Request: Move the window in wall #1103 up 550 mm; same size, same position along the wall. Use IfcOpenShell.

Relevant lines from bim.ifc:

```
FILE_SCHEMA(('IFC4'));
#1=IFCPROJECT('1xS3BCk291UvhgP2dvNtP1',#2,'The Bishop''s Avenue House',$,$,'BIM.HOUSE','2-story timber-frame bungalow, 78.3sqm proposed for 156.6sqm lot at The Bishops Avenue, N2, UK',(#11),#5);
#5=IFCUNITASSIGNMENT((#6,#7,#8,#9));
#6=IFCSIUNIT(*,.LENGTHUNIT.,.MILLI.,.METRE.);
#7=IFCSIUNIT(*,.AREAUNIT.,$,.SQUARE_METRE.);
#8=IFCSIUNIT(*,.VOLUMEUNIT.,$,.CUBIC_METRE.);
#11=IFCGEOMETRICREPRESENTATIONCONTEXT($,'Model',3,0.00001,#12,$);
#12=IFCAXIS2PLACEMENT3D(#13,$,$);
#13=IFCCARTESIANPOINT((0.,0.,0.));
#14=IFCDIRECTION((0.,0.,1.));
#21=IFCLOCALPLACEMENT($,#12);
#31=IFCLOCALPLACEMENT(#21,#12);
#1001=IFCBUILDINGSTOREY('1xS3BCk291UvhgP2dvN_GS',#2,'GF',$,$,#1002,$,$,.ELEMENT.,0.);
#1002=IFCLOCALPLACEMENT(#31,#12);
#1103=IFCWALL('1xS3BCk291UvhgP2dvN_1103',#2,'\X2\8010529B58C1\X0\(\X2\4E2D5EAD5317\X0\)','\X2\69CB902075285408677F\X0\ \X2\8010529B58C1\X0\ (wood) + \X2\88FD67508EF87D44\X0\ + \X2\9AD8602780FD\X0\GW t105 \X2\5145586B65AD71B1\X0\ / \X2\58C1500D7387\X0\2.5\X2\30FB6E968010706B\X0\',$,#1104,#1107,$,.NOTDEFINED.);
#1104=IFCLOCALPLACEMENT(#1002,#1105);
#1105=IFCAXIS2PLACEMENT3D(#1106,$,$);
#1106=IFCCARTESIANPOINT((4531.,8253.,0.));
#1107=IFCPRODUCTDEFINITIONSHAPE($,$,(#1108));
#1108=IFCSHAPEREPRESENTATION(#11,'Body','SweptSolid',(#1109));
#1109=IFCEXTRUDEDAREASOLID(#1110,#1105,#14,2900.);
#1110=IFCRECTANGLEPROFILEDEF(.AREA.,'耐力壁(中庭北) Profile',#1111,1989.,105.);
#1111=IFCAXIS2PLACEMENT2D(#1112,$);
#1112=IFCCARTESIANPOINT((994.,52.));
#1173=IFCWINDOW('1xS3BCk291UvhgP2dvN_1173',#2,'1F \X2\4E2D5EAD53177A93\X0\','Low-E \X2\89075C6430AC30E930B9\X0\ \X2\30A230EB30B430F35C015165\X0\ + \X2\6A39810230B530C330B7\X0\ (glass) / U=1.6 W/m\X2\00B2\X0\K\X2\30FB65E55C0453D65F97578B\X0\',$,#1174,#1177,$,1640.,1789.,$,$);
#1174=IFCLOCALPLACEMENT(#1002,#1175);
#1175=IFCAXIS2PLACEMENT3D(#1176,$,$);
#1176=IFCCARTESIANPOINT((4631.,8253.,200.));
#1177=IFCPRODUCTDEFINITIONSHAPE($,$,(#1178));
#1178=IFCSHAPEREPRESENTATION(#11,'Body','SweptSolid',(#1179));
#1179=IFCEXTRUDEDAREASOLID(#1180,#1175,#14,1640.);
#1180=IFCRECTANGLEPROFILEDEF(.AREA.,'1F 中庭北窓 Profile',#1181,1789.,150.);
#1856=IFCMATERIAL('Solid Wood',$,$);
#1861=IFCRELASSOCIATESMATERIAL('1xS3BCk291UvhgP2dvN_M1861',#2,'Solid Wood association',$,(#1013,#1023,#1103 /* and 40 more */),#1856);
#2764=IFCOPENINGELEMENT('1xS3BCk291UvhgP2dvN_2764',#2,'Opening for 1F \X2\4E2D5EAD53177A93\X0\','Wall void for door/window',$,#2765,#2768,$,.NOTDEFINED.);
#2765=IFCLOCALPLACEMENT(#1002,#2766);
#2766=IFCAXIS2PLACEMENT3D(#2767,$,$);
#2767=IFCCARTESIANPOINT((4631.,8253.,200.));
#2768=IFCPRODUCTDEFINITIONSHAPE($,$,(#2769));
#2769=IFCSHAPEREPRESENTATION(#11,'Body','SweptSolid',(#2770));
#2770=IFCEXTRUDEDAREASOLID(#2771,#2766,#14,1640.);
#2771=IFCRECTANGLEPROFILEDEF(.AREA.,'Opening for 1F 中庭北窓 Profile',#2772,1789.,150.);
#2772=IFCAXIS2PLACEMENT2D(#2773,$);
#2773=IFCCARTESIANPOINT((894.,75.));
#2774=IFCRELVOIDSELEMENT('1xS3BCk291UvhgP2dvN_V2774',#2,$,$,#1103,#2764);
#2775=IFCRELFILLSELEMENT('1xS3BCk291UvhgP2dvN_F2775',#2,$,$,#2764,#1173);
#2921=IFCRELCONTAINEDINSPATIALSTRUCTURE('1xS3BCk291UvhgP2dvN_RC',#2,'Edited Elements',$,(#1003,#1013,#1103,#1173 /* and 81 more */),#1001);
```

```python
import numpy as np
import ifcopenshell
import ifcopenshell.api.geometry
import ifcopenshell.util.placement
import ifcopenshell.util.unit

model = ifcopenshell.open("bim.ifc")
unit_scale = ifcopenshell.util.unit.calculate_unit_scale(model)

window = model.by_id(1173)
opening = window.FillsVoids[0].RelatingOpeningElement
dz = 550.0

shift = np.array([0.0, 0.0, dz])
# The window is not placed relative to its opening, so move both.
for product in (opening, window):
    matrix = ifcopenshell.util.placement.get_local_placement(product.ObjectPlacement)
    matrix[:3, 3] += shift
    ifcopenshell.api.geometry.edit_object_placement(model, product=product, matrix=matrix, is_si=False)

print(f"moved by {dz * unit_scale:+.3f} m")

model.write("bim-out.ifc")
```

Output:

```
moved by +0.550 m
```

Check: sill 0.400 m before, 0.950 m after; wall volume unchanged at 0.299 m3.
